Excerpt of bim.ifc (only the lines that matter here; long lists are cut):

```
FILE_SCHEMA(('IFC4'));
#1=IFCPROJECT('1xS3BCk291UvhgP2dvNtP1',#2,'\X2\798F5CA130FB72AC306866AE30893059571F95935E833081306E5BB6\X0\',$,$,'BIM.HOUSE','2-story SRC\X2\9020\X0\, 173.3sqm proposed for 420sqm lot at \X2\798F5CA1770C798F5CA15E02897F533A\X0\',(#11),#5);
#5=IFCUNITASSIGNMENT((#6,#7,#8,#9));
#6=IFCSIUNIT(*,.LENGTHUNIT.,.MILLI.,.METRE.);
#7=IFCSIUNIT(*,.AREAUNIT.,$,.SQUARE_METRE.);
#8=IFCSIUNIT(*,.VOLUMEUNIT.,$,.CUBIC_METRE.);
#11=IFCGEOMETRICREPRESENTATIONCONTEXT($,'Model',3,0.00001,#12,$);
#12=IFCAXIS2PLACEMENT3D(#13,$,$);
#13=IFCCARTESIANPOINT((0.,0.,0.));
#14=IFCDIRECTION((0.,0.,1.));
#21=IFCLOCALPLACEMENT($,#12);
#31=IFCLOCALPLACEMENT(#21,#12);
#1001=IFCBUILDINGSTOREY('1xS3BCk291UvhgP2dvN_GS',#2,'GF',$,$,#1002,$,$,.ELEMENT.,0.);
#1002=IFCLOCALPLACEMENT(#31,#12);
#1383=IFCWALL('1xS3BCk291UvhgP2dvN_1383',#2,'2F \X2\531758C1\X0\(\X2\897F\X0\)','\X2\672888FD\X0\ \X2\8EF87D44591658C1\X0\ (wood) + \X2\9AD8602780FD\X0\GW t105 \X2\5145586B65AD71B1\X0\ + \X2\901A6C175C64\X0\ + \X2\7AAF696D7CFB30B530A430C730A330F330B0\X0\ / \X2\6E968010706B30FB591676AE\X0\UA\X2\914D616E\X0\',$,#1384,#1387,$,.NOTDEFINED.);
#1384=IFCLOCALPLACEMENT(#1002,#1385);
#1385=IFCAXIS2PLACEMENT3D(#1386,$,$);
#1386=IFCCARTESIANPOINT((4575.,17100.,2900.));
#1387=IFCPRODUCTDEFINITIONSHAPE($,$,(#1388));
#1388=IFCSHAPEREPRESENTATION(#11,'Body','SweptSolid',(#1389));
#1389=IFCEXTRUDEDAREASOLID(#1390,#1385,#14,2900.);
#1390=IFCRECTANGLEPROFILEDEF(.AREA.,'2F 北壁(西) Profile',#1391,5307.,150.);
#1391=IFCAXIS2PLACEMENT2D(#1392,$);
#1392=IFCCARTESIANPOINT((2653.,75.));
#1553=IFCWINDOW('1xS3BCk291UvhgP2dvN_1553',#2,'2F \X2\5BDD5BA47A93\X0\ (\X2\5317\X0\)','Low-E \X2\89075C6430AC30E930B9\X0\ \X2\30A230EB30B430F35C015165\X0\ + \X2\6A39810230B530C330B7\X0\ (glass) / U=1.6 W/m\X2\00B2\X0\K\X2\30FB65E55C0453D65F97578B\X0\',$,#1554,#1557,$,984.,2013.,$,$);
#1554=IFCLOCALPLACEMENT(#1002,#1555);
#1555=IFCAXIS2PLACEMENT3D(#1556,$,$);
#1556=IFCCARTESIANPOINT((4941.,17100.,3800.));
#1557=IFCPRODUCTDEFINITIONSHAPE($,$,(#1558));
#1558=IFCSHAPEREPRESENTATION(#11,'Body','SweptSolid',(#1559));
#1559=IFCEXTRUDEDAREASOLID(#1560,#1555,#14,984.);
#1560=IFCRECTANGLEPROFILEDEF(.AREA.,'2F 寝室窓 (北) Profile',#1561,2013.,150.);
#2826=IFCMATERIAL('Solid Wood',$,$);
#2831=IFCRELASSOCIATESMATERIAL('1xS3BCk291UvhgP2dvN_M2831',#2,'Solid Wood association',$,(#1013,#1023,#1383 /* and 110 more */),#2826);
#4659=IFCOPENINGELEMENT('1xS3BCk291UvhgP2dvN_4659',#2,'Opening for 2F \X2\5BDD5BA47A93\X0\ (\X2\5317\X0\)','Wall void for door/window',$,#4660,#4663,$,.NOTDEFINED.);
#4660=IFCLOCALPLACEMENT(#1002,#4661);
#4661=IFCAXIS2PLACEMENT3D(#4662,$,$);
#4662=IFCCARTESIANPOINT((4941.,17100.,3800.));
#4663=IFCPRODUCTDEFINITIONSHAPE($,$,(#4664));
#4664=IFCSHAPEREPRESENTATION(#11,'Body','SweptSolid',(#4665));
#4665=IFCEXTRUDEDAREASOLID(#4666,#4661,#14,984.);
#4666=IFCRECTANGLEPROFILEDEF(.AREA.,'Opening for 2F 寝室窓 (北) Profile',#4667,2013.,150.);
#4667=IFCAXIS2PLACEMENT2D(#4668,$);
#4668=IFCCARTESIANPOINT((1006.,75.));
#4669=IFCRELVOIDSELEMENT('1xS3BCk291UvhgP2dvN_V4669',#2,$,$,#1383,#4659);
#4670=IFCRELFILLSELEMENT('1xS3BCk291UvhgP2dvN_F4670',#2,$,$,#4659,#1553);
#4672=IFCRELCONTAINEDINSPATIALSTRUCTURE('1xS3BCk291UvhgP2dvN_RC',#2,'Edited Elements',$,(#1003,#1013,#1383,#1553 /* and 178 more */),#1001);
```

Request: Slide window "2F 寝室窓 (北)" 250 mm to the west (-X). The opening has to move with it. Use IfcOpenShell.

```python
import ifcopenshell
import ifcopenshell.api.geometry
import ifcopenshell.util.placement

model = ifcopenshell.open("bim.ifc")

window = model.by_id(1553)
opening = window.FillsVoids[0].RelatingOpeningElement
wall = opening.VoidsElements[0].RelatingBuildingElement

wall_matrix = ifcopenshell.util.placement.get_local_placement(wall.ObjectPlacement)
shift = wall_matrix[:3, 0] * -250.0
before = ifcopenshell.util.placement.get_local_placement(window.ObjectPlacement)[:3, 3].copy()

# The window is not placed relative to its opening, so move both.
for product in (opening, window):
    matrix = ifcopenshell.util.placement.get_local_placement(product.ObjectPlacement)
    matrix[:3, 3] += shift
    ifcopenshell.api.geometry.edit_object_placement(model, product=product, matrix=matrix, is_si=False)

after = ifcopenshell.util.placement.get_local_placement(window.ObjectPlacement)[:3, 3]
print("window moved by", (after - before).round(3) + 0.0)

model.write("bim-out.ifc")
```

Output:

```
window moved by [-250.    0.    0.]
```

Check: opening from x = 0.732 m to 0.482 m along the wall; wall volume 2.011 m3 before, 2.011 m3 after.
